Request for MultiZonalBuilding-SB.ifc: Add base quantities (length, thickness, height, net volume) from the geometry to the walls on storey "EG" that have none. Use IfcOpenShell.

First a look at what the model holds.

```python
import ifcopenshell
import ifcopenshell.util.element
import ifcopenshell.util.unit

model = ifcopenshell.open("MultiZonalBuilding-SB.ifc")
print(model.schema)
for unit_type in ("LENGTHUNIT", "AREAUNIT", "VOLUMEUNIT"):
    print(unit_type, ifcopenshell.util.unit.calculate_unit_scale(model, unit_type))
storey = next(s for s in model.by_type("IfcBuildingStorey") if s.Name == "EG")
walls = [e for e in ifcopenshell.util.element.get_decomposition(storey) if e.is_a("IfcWall")]
for e in sorted(walls, key=lambda e: e.id()):
    print(e.id(), e.is_a(), e.Name, list(ifcopenshell.util.element.get_psets(e, qtos_only=True)), sep=" | ")
```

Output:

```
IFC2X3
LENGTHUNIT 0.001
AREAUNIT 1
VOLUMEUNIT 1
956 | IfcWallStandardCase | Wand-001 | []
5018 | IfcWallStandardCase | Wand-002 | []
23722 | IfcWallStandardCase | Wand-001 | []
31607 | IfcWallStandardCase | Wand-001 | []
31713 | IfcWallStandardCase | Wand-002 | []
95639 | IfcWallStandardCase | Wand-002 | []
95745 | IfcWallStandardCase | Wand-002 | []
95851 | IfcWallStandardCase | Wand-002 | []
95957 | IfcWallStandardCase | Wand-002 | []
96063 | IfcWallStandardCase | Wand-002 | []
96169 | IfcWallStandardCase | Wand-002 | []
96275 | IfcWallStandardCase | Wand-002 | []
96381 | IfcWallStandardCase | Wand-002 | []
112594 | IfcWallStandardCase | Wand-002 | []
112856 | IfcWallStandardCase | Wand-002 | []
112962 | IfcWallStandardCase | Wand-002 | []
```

```python
import ifcopenshell
import ifcopenshell.api.pset
import ifcopenshell.geom
import ifcopenshell.util.element
import ifcopenshell.util.shape
import ifcopenshell.util.unit

model = ifcopenshell.open("MultiZonalBuilding-SB.ifc")
unit_scale = ifcopenshell.util.unit.calculate_unit_scale(model)
volume_scale = ifcopenshell.util.unit.calculate_unit_scale(model, "VOLUMEUNIT")
settings = ifcopenshell.geom.settings()

storey = next(s for s in model.by_type("IfcBuildingStorey") if s.Name == "EG")
walls = [e for e in ifcopenshell.util.element.get_decomposition(storey) if e.is_a("IfcWall")]

for e in sorted(walls, key=lambda e: e.id()):
    if ifcopenshell.util.element.get_psets(e, qtos_only=True, should_inherit=False):
        continue
    # Geometry comes back in metres, in the element's own axes.
    shape = ifcopenshell.geom.create_shape(settings, e)
    values = {
        "Length": ifcopenshell.util.shape.get_x(shape.geometry) / unit_scale,
        "Width": ifcopenshell.util.shape.get_y(shape.geometry) / unit_scale,
        "Height": ifcopenshell.util.shape.get_z(shape.geometry) / unit_scale,
        "NetVolume": ifcopenshell.util.shape.get_volume(shape.geometry) / volume_scale,
    }
    qto = ifcopenshell.api.pset.add_qto(model, product=e, name="BaseQuantities")
    ifcopenshell.api.pset.edit_qto(model, qto=qto, properties=values)
    print(e.id(), {k: round(v, 3) for k, v in values.items()})

model.write("MultiZonalBuilding-SB_rev.ifc")
```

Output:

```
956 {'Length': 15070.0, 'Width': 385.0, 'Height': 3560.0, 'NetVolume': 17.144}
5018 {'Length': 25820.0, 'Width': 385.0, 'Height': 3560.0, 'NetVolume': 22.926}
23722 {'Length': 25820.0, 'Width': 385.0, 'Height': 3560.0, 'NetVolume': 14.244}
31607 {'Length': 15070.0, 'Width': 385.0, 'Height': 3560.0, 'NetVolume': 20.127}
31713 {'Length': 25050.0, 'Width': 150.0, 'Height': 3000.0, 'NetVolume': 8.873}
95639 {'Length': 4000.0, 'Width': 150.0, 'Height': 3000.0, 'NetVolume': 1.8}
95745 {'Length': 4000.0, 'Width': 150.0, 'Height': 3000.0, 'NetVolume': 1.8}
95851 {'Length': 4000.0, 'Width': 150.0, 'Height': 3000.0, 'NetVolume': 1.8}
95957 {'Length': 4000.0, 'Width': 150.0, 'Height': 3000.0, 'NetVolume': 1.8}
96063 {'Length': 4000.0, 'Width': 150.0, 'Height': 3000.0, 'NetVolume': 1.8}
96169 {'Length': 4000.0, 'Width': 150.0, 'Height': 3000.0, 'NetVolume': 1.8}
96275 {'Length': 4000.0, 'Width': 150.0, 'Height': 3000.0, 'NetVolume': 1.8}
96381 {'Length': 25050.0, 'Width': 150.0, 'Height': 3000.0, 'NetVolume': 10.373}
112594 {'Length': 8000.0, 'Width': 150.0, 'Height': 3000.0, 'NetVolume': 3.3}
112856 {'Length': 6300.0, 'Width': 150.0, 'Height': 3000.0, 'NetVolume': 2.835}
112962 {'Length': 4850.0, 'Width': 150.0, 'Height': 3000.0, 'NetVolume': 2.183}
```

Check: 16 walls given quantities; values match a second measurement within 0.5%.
